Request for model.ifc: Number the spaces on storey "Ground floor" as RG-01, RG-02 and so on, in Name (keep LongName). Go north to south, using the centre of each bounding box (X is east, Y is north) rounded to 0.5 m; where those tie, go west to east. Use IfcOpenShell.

First a look at what the model holds.

```python
import ifcopenshell
import ifcopenshell.util.element
import ifcopenshell.util.placement

model = ifcopenshell.open("model.ifc")
print(model.schema)
storey = next(s for s in model.by_type("IfcBuildingStorey") if s.Name == "Ground floor")
spaces = [e for e in ifcopenshell.util.element.get_decomposition(storey) if e.is_a("IfcSpace")]
for e in sorted(spaces, key=lambda e: e.id()):
    origin = ifcopenshell.util.placement.get_local_placement(e.ObjectPlacement)[:3, 3]
    print(e.id(), e.Name, e.LongName, origin.round(2) + 0.0, sep=" | ")
```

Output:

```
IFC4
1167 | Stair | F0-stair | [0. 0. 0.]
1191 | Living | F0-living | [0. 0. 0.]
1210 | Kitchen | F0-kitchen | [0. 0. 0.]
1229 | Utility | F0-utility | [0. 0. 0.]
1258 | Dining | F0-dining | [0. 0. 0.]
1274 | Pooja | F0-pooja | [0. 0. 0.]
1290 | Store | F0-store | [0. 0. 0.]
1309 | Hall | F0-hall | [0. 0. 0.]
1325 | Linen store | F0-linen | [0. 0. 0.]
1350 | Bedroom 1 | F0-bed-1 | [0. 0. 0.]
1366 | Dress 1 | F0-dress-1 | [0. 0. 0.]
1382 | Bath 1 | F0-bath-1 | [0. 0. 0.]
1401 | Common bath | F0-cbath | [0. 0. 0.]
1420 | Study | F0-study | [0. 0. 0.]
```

```python
import ifcopenshell
import ifcopenshell.geom
import ifcopenshell.util.element
import ifcopenshell.util.shape

model = ifcopenshell.open("model.ifc")
settings = ifcopenshell.geom.settings()
settings.set("use-world-coords", True)


def centre(element):
    shape = ifcopenshell.geom.create_shape(settings, element)
    return ifcopenshell.util.shape.get_bbox_centroid(shape.geometry)


storey = next(s for s in model.by_type("IfcBuildingStorey") if s.Name == "Ground floor")
spaces = [e for e in ifcopenshell.util.element.get_decomposition(storey) if e.is_a("IfcSpace")]

# Insertion points can sit at a corner or the storey origin, so sort by the geometry (in metres).
centres = {e: centre(e) for e in spaces}
spaces.sort(key=lambda e: (-round(centres[e][1] / 0.5), centres[e][0]))

for i, e in enumerate(spaces, start=1):
    number = f"RG-{i:02d}"
    e.Name = number
    print(e.id(), number)

model.write("model_rev.ifc")
```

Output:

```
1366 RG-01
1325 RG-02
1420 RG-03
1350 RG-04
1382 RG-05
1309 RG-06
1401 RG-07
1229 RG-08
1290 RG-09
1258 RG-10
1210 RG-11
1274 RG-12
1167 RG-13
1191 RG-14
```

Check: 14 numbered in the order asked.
